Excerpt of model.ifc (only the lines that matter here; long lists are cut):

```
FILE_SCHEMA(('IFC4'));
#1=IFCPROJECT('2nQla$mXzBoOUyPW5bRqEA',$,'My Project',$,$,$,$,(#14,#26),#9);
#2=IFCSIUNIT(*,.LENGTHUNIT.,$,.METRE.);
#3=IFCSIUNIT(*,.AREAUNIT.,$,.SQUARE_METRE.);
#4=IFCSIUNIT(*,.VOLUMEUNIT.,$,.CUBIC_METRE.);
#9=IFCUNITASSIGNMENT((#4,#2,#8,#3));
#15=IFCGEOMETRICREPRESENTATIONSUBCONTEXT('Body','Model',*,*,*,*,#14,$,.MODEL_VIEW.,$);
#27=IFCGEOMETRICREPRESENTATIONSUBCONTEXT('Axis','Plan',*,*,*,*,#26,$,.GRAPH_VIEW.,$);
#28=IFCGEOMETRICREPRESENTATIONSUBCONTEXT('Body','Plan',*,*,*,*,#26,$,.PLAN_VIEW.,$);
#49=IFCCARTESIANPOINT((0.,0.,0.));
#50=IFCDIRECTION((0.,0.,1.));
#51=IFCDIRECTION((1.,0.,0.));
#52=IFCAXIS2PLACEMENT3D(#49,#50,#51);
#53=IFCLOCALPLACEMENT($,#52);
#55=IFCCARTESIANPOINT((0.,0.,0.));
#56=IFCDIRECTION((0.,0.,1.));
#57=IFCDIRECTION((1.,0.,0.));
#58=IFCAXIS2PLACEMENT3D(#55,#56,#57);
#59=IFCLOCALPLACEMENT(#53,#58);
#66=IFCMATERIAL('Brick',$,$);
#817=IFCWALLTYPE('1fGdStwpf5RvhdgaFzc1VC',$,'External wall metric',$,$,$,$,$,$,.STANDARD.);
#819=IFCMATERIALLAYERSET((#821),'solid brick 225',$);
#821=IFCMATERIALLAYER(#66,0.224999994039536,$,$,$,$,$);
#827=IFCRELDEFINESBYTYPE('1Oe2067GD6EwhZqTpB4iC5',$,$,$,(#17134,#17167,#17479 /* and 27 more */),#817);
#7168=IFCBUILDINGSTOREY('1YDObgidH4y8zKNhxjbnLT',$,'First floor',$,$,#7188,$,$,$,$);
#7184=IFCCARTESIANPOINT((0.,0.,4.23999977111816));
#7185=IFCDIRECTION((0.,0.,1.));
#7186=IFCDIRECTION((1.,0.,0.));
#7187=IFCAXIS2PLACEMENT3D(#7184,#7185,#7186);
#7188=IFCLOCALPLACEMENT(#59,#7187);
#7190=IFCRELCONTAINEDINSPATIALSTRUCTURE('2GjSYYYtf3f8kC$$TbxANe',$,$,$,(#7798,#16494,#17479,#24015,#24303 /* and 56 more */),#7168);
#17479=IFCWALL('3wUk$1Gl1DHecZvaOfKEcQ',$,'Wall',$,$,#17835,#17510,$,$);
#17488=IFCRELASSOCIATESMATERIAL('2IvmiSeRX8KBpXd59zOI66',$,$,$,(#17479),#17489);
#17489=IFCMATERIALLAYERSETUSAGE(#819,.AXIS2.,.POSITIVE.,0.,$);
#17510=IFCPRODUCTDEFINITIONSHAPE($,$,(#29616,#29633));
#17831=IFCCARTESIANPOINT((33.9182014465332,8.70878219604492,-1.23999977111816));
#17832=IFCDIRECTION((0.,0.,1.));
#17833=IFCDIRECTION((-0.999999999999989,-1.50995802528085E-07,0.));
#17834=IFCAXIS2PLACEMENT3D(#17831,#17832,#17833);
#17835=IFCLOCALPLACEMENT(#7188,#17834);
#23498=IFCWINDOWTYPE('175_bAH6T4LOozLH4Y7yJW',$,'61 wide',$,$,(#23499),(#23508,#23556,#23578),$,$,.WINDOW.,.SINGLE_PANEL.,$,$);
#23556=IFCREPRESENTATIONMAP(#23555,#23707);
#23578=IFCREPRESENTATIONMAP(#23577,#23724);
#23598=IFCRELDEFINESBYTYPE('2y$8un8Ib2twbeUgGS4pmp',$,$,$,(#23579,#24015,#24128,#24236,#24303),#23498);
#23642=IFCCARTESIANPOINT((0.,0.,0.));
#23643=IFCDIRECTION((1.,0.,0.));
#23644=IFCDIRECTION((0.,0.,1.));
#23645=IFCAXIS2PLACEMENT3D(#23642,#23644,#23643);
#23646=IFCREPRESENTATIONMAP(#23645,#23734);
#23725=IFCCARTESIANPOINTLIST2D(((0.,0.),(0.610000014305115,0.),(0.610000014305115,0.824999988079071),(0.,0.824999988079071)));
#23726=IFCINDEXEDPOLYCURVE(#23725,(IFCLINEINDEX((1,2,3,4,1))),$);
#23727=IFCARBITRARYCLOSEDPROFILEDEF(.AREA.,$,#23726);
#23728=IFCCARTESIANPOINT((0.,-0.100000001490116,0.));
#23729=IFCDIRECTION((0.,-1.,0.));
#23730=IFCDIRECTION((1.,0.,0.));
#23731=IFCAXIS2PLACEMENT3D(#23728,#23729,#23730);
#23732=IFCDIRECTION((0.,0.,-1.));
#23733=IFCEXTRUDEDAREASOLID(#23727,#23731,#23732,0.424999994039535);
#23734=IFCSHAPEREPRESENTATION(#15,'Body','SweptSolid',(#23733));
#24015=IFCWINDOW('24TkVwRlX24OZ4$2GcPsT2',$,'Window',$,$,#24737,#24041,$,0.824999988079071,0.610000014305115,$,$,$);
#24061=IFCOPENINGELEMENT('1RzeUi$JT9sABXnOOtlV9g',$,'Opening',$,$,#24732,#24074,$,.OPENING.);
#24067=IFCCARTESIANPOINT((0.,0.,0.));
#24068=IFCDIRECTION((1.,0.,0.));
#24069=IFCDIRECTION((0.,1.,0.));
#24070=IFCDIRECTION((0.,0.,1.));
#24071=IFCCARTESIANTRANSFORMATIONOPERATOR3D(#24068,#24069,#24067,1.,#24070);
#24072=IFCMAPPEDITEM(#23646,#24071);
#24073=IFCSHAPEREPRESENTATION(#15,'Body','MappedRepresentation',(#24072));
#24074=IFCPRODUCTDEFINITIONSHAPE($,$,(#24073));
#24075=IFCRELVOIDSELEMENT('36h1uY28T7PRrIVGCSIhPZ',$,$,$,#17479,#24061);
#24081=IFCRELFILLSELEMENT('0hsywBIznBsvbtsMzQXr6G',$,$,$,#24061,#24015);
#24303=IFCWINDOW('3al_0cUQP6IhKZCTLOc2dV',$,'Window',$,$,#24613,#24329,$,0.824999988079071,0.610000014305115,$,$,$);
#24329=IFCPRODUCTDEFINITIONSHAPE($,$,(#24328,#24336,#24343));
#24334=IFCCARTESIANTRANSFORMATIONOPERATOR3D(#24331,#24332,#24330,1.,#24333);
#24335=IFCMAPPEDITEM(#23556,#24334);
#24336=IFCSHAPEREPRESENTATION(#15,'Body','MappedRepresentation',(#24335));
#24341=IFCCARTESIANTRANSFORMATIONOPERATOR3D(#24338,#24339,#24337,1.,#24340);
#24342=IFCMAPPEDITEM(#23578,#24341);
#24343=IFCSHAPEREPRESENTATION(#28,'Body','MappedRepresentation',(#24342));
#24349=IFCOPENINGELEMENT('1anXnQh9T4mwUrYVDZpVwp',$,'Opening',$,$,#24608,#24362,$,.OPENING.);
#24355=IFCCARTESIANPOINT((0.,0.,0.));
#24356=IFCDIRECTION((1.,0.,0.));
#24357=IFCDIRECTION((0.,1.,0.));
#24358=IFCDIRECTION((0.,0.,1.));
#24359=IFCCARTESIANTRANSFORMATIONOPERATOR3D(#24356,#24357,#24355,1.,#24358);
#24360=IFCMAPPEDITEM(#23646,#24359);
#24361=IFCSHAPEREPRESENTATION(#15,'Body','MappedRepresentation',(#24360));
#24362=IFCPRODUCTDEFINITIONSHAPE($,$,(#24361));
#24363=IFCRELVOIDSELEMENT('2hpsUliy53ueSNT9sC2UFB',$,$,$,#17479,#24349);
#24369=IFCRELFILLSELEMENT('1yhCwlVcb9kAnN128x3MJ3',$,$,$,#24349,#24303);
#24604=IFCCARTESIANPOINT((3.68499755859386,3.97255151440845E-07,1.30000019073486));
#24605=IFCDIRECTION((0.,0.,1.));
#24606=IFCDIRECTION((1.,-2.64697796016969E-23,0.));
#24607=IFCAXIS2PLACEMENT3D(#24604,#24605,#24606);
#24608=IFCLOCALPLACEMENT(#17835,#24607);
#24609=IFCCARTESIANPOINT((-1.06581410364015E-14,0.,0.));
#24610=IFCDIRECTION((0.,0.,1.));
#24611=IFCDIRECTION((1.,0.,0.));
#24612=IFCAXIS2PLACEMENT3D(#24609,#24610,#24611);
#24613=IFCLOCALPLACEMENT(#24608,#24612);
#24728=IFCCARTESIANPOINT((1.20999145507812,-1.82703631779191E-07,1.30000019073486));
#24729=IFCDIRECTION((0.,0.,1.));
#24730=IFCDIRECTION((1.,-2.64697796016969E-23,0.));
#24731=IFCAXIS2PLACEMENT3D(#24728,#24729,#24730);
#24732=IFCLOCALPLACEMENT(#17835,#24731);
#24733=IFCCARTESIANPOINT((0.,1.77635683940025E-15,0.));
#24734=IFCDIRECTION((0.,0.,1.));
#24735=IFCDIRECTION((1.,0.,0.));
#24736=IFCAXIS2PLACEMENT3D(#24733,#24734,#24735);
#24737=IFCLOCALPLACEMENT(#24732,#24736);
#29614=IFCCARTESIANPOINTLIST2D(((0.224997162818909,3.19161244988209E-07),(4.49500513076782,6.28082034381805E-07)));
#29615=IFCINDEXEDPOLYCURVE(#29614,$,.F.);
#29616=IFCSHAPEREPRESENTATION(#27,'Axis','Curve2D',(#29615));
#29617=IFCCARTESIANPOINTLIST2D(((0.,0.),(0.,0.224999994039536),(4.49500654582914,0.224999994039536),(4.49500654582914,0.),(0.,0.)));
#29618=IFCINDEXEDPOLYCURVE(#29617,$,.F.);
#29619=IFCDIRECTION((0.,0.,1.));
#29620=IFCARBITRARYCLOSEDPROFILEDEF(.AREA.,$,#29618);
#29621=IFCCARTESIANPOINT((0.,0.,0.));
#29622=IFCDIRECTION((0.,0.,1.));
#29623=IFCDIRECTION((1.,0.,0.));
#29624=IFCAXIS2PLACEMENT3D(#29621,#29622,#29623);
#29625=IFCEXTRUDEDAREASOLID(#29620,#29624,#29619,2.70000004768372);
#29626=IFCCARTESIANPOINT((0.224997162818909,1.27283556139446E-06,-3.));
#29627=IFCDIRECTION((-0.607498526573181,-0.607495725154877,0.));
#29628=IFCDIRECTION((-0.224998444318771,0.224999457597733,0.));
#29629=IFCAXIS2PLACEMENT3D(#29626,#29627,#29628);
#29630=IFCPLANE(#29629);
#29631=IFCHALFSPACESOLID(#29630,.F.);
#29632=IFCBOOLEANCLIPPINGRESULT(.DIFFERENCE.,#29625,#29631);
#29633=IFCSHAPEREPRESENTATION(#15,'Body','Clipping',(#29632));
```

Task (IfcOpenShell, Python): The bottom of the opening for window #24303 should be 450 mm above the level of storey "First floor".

```python
import numpy as np
import ifcopenshell
import ifcopenshell.api.geometry
import ifcopenshell.geom
import ifcopenshell.util.element
import ifcopenshell.util.placement
import ifcopenshell.util.shape
import ifcopenshell.util.unit

model = ifcopenshell.open("model.ifc")
unit_scale = ifcopenshell.util.unit.calculate_unit_scale(model)

window = model.by_guid("3al_0cUQP6IhKZCTLOc2dV")
opening = window.FillsVoids[0].RelatingOpeningElement
storey = ifcopenshell.util.element.get_container(window, ifc_class="IfcBuildingStorey")
level = ifcopenshell.util.placement.get_local_placement(storey.ObjectPlacement)[2, 3]

# The opening's origin need not be at the sill, so measure its lowest point.
shape = ifcopenshell.geom.create_shape(ifcopenshell.geom.settings(), opening)
bottom = ifcopenshell.util.shape.get_shape_bottom_elevation(shape, shape.geometry) / unit_scale
dz = level + 0.45 / unit_scale - bottom

shift = np.array([0.0, 0.0, dz])
# The window is placed relative to its opening, so it follows when the opening moves.
matrix = ifcopenshell.util.placement.get_local_placement(opening.ObjectPlacement)
matrix[:3, 3] += shift
ifcopenshell.api.geometry.edit_object_placement(
    model, product=opening, matrix=matrix, is_si=False, should_transform_children=True
)

print(f"moved by {dz * unit_scale:+.3f} m")

model.write("model_v2.ifc")
```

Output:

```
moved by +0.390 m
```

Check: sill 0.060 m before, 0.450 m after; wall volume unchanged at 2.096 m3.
